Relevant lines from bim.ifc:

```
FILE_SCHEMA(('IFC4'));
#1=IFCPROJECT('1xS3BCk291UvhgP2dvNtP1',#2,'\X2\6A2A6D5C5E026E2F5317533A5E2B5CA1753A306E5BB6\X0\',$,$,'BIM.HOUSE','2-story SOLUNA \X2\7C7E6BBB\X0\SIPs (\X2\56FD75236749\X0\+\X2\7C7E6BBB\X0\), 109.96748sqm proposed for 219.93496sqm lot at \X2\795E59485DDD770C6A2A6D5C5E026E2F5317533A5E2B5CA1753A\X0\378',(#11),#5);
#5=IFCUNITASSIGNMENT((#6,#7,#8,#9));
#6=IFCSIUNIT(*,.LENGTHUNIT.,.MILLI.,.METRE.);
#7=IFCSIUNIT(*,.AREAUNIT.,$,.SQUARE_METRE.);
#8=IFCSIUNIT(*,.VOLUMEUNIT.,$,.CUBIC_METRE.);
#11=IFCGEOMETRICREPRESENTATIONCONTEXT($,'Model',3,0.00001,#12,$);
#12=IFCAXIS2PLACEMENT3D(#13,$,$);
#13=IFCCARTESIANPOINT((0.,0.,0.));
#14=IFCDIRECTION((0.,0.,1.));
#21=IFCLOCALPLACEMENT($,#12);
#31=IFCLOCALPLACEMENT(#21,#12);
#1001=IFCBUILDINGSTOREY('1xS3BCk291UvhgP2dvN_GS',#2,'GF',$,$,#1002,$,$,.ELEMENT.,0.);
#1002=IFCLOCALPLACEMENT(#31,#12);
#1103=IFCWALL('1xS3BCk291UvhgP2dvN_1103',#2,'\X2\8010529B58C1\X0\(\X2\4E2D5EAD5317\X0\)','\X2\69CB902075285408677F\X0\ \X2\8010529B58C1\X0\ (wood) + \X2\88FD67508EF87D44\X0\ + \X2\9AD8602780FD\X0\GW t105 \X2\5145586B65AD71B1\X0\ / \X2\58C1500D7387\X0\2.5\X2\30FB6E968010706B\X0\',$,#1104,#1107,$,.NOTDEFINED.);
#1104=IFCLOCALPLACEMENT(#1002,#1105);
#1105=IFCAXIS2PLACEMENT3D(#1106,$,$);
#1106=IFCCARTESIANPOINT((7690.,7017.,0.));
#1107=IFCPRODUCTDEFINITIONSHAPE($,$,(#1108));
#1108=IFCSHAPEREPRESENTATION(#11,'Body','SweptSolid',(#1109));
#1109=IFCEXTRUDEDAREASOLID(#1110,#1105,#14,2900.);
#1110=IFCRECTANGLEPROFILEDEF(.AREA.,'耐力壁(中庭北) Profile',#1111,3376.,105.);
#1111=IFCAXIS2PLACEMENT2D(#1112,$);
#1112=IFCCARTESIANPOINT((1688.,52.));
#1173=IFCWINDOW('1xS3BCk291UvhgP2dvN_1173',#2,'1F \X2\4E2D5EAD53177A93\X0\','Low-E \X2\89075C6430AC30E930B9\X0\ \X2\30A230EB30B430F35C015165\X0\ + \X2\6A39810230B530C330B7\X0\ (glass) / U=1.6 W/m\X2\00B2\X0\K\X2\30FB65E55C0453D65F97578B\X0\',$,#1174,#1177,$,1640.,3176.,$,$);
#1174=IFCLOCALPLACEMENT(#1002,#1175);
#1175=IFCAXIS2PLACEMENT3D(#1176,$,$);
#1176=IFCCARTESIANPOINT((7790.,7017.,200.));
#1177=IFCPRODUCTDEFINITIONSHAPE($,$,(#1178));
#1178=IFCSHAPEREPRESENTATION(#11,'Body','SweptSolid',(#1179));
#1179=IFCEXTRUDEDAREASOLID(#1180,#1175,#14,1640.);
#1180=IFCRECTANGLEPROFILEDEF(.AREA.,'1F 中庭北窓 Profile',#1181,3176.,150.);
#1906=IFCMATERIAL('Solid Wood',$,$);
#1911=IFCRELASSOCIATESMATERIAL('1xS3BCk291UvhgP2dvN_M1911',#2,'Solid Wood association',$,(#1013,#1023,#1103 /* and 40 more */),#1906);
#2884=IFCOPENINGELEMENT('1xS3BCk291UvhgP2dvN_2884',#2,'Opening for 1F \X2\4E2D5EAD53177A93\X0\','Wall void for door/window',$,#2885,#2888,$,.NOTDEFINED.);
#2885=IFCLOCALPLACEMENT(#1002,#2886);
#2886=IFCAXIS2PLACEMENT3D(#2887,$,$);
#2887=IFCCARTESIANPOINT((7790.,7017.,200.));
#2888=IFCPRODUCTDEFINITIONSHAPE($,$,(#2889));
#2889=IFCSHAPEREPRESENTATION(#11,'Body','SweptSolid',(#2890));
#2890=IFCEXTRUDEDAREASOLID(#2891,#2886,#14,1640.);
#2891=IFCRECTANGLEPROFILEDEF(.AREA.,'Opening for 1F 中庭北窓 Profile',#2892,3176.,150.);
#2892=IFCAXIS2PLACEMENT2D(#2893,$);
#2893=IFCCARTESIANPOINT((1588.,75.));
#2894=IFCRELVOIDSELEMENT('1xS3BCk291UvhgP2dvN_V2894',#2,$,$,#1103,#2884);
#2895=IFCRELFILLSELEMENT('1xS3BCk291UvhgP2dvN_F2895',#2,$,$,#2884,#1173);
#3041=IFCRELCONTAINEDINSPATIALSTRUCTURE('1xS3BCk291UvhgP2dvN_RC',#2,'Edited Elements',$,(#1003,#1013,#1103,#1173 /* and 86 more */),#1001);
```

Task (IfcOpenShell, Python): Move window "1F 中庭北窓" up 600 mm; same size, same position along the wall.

```python
import numpy as np
import ifcopenshell
import ifcopenshell.api.geometry
import ifcopenshell.util.placement
import ifcopenshell.util.unit

model = ifcopenshell.open("bim.ifc")
unit_scale = ifcopenshell.util.unit.calculate_unit_scale(model)

window = model.by_guid("1xS3BCk291UvhgP2dvN_1173")
opening = window.FillsVoids[0].RelatingOpeningElement
dz = 0.6 / unit_scale

shift = np.array([0.0, 0.0, dz])
# The window is not placed relative to its opening, so move both.
for product in (opening, window):
    matrix = ifcopenshell.util.placement.get_local_placement(product.ObjectPlacement)
    matrix[:3, 3] += shift
    ifcopenshell.api.geometry.edit_object_placement(model, product=product, matrix=matrix, is_si=False)

print(f"moved by {dz * unit_scale:+.3f} m")

model.write("bim_v2.ifc")
```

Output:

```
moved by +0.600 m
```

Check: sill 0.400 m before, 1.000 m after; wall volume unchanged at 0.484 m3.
